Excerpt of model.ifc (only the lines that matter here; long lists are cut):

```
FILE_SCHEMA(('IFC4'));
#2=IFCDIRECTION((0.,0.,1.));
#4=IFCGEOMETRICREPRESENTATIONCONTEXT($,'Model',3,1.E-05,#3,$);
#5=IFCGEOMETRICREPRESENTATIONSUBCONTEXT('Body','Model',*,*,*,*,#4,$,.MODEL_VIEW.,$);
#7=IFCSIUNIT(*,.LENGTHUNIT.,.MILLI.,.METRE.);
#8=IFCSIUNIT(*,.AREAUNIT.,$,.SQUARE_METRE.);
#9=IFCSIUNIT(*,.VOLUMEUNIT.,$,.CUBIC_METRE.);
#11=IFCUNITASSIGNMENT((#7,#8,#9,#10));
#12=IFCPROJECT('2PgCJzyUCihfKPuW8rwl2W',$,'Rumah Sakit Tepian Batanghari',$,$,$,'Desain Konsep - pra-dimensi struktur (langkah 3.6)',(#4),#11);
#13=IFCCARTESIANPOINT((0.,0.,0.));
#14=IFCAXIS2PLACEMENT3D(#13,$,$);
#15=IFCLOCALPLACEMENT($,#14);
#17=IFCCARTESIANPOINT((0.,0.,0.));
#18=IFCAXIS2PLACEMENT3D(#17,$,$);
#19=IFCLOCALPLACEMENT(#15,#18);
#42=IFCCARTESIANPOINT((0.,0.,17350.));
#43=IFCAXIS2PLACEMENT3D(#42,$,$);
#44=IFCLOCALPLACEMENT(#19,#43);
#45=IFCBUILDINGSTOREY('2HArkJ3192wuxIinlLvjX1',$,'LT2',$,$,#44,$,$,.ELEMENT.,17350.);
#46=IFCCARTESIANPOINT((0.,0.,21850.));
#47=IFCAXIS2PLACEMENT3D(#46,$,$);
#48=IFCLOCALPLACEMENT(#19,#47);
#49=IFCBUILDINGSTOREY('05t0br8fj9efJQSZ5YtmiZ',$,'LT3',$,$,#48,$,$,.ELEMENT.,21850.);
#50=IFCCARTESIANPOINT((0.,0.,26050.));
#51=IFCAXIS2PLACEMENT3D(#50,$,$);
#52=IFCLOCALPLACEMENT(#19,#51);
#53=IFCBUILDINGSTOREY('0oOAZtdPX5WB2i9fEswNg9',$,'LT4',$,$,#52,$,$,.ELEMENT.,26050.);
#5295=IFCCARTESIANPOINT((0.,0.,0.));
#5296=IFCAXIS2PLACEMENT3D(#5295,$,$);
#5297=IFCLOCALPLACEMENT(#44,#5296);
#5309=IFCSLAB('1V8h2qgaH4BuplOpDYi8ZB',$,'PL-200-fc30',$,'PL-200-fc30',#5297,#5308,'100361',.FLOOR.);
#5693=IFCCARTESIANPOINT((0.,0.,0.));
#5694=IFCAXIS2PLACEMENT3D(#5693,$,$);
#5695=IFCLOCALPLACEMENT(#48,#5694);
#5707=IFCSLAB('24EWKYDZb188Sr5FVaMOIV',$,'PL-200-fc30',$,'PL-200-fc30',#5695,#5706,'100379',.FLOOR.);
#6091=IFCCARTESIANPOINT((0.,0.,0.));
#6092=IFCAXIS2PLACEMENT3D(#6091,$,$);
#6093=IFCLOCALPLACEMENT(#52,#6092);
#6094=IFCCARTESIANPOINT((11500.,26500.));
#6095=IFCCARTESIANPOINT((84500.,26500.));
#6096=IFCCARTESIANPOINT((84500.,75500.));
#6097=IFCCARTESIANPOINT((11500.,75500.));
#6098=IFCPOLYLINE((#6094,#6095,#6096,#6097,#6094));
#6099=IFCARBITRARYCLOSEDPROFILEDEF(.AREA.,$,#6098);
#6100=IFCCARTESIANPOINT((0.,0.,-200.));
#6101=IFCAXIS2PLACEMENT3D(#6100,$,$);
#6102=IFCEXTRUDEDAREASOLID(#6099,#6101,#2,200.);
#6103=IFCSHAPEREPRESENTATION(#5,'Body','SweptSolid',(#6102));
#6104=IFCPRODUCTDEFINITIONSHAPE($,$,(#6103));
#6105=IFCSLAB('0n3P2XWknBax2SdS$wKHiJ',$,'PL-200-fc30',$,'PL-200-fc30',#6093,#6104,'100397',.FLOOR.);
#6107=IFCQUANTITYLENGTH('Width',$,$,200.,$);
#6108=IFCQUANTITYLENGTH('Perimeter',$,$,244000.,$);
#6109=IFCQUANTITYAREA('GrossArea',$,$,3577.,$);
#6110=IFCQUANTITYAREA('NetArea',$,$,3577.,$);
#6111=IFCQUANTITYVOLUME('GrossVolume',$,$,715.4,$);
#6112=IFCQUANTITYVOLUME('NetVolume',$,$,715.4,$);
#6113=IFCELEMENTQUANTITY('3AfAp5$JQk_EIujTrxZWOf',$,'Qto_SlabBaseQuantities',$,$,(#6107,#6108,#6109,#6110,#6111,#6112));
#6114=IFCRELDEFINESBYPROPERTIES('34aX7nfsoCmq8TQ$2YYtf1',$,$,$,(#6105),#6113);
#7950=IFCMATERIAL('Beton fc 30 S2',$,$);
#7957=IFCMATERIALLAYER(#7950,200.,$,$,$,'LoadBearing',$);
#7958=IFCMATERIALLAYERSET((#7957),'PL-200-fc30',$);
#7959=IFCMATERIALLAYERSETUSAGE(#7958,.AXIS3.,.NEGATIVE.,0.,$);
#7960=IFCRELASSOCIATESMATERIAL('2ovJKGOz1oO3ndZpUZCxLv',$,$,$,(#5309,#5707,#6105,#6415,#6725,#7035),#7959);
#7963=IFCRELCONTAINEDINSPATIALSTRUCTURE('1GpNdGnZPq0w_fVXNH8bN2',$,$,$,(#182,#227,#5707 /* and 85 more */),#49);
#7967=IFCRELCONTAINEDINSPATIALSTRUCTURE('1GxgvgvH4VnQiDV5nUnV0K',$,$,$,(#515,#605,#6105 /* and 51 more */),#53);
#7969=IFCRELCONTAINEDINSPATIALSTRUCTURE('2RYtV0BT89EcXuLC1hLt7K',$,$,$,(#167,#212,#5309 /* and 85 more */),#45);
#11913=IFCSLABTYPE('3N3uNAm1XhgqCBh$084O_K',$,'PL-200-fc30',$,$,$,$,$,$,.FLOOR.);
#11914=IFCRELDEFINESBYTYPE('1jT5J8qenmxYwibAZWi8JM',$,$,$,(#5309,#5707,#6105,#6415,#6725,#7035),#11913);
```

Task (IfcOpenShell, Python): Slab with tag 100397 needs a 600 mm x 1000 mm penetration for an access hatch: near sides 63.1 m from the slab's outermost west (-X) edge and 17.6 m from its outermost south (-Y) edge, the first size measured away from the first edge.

```python
import numpy as np
import ifcopenshell
import ifcopenshell.api.feature
import ifcopenshell.api.geometry
import ifcopenshell.api.pset
import ifcopenshell.api.root
import ifcopenshell.geom
import ifcopenshell.util.element
import ifcopenshell.util.placement
import ifcopenshell.util.representation
import ifcopenshell.util.shape
import ifcopenshell.util.unit

model = ifcopenshell.open("model.ifc")
unit_scale = ifcopenshell.util.unit.calculate_unit_scale(model)
area_scale = ifcopenshell.util.unit.calculate_unit_scale(model, "AREAUNIT")
volume_scale = ifcopenshell.util.unit.calculate_unit_scale(model, "VOLUMEUNIT")
settings = ifcopenshell.geom.settings()


def volume(element):
    """Net volume in cubic metres, openings subtracted."""
    shape = ifcopenshell.geom.create_shape(settings, element)
    return ifcopenshell.util.shape.get_volume(shape.geometry)


slab = model.by_id(6105)
before = volume(slab)

# Extent in the slab's own axes, in metres. The edges named are its -X and -Y sides.
slab_shape = ifcopenshell.geom.create_shape(settings, slab)
vertices = ifcopenshell.util.shape.get_vertices(slab_shape.geometry)
x_min, y_min, bottom = vertices.min(axis=0)
top = vertices[:, 2].max()

opening = ifcopenshell.api.root.create_entity(model, ifc_class="IfcOpeningElement", name="Access hatch opening", predefined_type="OPENING")
context = ifcopenshell.util.representation.get_context(model, "Model", "Body", "MODEL_VIEW")
width, depth = 0.6, 1
outline = [(0.0, 0.0), (width, 0.0), (width, depth), (0.0, depth), (0.0, 0.0)]
# Overshoot both faces by 50 mm so the cut is clean.
shape = ifcopenshell.api.geometry.add_slab_representation(
    model, context=context, depth=top - bottom + 0.1, polyline=outline
)
ifcopenshell.api.geometry.assign_representation(model, product=opening, representation=shape)

matrix = ifcopenshell.util.placement.get_local_placement(slab.ObjectPlacement)
matrix[:, 3] = matrix @ np.append(np.array([x_min + 63.1, y_min + 17.6, bottom - 0.05]) / unit_scale, 1.0)
ifcopenshell.api.geometry.edit_object_placement(model, product=opening, matrix=matrix, is_si=False)
ifcopenshell.api.feature.add_feature(model, feature=opening, element=slab)

after = volume(slab)

# Update the slab's stored quantities.
qto = model.by_id(ifcopenshell.util.element.get_pset(slab, "Qto_SlabBaseQuantities", should_inherit=False)["id"])
ifcopenshell.api.pset.edit_qto(model, qto=qto, properties={
    "NetArea": after / (top - bottom) / area_scale,
    "NetVolume": after / volume_scale,
})

print(f"slab volume {before:.3f} -> {after:.3f} m3")

model.write("model_updated.ifc")
```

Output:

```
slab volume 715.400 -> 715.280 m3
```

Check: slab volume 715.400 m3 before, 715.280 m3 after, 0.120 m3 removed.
